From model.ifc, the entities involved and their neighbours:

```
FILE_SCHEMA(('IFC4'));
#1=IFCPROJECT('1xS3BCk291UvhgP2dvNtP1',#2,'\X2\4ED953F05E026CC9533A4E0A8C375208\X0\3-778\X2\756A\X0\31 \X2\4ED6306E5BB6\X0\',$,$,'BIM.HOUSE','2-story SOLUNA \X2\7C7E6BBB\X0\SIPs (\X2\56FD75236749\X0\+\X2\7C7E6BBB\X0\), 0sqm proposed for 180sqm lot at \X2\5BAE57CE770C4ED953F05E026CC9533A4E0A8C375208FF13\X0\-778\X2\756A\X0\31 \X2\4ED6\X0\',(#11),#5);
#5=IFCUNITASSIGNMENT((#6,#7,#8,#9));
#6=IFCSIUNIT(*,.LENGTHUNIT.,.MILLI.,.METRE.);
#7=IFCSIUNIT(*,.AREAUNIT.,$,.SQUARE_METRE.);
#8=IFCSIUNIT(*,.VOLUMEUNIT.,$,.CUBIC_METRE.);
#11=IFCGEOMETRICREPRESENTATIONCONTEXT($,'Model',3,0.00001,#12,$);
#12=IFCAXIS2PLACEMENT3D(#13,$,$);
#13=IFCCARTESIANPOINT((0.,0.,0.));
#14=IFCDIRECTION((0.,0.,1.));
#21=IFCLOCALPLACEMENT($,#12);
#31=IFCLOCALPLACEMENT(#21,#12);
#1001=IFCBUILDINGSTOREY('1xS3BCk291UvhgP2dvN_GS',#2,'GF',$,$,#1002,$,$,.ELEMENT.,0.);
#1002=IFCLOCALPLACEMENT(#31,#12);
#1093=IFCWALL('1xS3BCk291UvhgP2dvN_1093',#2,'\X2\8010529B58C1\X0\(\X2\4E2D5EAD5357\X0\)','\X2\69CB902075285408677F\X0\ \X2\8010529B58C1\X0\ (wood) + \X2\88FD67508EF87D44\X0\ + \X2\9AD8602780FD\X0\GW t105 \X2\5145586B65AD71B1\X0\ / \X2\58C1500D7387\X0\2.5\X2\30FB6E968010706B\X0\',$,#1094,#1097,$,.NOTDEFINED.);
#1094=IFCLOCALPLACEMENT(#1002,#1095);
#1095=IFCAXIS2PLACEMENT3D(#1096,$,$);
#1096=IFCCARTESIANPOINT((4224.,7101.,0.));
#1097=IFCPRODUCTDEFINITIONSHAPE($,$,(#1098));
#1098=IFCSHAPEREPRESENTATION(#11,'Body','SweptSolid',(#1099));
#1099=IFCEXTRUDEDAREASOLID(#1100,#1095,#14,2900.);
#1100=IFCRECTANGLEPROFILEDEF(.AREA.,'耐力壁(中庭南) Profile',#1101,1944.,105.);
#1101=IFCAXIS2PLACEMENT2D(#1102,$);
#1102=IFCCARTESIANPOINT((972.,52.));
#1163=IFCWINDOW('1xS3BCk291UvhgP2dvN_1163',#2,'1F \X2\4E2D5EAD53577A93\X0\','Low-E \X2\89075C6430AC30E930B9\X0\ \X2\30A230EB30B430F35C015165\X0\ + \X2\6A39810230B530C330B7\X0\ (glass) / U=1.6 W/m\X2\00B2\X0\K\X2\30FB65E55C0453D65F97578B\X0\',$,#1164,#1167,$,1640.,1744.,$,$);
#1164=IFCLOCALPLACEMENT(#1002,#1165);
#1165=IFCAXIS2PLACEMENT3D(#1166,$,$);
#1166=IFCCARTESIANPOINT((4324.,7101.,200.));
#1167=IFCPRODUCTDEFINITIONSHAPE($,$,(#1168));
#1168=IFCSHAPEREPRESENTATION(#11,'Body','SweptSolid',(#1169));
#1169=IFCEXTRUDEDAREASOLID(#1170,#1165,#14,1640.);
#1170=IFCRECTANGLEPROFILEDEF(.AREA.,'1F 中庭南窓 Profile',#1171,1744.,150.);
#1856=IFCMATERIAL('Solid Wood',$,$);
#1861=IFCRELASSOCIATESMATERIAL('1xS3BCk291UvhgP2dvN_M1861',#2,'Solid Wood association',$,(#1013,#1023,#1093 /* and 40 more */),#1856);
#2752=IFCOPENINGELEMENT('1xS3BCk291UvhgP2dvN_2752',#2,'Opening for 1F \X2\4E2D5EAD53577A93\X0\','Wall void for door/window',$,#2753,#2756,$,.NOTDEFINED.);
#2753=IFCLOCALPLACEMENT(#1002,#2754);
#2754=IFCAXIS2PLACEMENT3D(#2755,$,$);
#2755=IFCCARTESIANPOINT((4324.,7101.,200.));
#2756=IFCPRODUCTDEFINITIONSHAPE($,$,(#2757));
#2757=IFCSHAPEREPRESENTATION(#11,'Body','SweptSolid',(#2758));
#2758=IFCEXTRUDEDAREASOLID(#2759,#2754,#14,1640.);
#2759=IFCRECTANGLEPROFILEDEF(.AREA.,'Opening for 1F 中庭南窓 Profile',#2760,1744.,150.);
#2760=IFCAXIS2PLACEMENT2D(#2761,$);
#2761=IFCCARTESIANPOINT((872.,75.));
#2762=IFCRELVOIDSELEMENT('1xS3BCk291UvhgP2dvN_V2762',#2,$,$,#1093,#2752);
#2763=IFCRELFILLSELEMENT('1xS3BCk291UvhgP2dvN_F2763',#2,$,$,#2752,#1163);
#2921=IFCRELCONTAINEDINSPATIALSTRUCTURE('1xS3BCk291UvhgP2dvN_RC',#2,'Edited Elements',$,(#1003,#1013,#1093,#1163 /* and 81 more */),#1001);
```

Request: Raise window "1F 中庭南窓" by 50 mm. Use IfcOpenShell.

```python
import numpy as np
import ifcopenshell
import ifcopenshell.api.geometry
import ifcopenshell.util.placement
import ifcopenshell.util.unit

model = ifcopenshell.open("model.ifc")
unit_scale = ifcopenshell.util.unit.calculate_unit_scale(model)

window = model.by_guid("1xS3BCk291UvhgP2dvN_1163")
opening = window.FillsVoids[0].RelatingOpeningElement
dz = 50.0

shift = np.array([0.0, 0.0, dz])
# The window is not placed relative to its opening, so move both.
for product in (opening, window):
    matrix = ifcopenshell.util.placement.get_local_placement(product.ObjectPlacement)
    matrix[:3, 3] += shift
    ifcopenshell.api.geometry.edit_object_placement(model, product=product, matrix=matrix, is_si=False)

print(f"moved by {dz * unit_scale:+.3f} m")

model.write("model_edited.ifc")
```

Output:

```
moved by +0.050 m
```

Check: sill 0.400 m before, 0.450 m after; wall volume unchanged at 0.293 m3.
